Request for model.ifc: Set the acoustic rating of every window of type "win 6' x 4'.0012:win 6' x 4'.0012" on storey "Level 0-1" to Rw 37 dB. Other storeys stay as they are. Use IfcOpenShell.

First a look at what the model holds.

```python
import ifcopenshell
import ifcopenshell.util.element

model = ifcopenshell.open("model.ifc")
print(model.schema)
storey = next(s for s in model.by_type("IfcBuildingStorey") if s.Name == "Level 0-1")
windows = [e for e in ifcopenshell.util.element.get_decomposition(storey) if e.is_a("IfcWindow")]
seen = {}
for e in windows:
    element_type = ifcopenshell.util.element.get_type(e)
    key = (element_type.Name if element_type != e and element_type else None, ifcopenshell.util.element.get_pset(e, "Pset_WindowCommon", "AcousticRating"))
    seen[key] = seen.get(key, 0) + 1
for (name, value), count in sorted(seen.items(), key=str):
    print(count, "x", name, "|", value)
```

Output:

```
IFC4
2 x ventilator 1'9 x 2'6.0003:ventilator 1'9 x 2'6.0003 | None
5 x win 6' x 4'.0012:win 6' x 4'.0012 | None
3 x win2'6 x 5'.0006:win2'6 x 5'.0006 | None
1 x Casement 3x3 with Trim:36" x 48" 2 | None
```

```python
import ifcopenshell
import ifcopenshell.api.pset
import ifcopenshell.util.element

model = ifcopenshell.open("model.ifc")

storey = next(s for s in model.by_type("IfcBuildingStorey") if s.Name == "Level 0-1")
windows = [e for e in ifcopenshell.util.element.get_decomposition(storey) if e.is_a("IfcWindow")]

count = 0
for e in windows:
    element_type = ifcopenshell.util.element.get_type(e)
    if element_type in (None, e) or element_type.Name != "win 6' x 4'.0012:win 6' x 4'.0012":
        continue
    # add_pset returns the element's existing set when there is one.
    pset = ifcopenshell.api.pset.add_pset(model, product=e, name="Pset_WindowCommon")
    ifcopenshell.api.pset.edit_pset(model, pset=pset, properties={"AcousticRating": "Rw 37 dB"})
    count += 1

print(count, "windows updated")

model.write("model_rev.ifc")
```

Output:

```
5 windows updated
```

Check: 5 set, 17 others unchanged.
